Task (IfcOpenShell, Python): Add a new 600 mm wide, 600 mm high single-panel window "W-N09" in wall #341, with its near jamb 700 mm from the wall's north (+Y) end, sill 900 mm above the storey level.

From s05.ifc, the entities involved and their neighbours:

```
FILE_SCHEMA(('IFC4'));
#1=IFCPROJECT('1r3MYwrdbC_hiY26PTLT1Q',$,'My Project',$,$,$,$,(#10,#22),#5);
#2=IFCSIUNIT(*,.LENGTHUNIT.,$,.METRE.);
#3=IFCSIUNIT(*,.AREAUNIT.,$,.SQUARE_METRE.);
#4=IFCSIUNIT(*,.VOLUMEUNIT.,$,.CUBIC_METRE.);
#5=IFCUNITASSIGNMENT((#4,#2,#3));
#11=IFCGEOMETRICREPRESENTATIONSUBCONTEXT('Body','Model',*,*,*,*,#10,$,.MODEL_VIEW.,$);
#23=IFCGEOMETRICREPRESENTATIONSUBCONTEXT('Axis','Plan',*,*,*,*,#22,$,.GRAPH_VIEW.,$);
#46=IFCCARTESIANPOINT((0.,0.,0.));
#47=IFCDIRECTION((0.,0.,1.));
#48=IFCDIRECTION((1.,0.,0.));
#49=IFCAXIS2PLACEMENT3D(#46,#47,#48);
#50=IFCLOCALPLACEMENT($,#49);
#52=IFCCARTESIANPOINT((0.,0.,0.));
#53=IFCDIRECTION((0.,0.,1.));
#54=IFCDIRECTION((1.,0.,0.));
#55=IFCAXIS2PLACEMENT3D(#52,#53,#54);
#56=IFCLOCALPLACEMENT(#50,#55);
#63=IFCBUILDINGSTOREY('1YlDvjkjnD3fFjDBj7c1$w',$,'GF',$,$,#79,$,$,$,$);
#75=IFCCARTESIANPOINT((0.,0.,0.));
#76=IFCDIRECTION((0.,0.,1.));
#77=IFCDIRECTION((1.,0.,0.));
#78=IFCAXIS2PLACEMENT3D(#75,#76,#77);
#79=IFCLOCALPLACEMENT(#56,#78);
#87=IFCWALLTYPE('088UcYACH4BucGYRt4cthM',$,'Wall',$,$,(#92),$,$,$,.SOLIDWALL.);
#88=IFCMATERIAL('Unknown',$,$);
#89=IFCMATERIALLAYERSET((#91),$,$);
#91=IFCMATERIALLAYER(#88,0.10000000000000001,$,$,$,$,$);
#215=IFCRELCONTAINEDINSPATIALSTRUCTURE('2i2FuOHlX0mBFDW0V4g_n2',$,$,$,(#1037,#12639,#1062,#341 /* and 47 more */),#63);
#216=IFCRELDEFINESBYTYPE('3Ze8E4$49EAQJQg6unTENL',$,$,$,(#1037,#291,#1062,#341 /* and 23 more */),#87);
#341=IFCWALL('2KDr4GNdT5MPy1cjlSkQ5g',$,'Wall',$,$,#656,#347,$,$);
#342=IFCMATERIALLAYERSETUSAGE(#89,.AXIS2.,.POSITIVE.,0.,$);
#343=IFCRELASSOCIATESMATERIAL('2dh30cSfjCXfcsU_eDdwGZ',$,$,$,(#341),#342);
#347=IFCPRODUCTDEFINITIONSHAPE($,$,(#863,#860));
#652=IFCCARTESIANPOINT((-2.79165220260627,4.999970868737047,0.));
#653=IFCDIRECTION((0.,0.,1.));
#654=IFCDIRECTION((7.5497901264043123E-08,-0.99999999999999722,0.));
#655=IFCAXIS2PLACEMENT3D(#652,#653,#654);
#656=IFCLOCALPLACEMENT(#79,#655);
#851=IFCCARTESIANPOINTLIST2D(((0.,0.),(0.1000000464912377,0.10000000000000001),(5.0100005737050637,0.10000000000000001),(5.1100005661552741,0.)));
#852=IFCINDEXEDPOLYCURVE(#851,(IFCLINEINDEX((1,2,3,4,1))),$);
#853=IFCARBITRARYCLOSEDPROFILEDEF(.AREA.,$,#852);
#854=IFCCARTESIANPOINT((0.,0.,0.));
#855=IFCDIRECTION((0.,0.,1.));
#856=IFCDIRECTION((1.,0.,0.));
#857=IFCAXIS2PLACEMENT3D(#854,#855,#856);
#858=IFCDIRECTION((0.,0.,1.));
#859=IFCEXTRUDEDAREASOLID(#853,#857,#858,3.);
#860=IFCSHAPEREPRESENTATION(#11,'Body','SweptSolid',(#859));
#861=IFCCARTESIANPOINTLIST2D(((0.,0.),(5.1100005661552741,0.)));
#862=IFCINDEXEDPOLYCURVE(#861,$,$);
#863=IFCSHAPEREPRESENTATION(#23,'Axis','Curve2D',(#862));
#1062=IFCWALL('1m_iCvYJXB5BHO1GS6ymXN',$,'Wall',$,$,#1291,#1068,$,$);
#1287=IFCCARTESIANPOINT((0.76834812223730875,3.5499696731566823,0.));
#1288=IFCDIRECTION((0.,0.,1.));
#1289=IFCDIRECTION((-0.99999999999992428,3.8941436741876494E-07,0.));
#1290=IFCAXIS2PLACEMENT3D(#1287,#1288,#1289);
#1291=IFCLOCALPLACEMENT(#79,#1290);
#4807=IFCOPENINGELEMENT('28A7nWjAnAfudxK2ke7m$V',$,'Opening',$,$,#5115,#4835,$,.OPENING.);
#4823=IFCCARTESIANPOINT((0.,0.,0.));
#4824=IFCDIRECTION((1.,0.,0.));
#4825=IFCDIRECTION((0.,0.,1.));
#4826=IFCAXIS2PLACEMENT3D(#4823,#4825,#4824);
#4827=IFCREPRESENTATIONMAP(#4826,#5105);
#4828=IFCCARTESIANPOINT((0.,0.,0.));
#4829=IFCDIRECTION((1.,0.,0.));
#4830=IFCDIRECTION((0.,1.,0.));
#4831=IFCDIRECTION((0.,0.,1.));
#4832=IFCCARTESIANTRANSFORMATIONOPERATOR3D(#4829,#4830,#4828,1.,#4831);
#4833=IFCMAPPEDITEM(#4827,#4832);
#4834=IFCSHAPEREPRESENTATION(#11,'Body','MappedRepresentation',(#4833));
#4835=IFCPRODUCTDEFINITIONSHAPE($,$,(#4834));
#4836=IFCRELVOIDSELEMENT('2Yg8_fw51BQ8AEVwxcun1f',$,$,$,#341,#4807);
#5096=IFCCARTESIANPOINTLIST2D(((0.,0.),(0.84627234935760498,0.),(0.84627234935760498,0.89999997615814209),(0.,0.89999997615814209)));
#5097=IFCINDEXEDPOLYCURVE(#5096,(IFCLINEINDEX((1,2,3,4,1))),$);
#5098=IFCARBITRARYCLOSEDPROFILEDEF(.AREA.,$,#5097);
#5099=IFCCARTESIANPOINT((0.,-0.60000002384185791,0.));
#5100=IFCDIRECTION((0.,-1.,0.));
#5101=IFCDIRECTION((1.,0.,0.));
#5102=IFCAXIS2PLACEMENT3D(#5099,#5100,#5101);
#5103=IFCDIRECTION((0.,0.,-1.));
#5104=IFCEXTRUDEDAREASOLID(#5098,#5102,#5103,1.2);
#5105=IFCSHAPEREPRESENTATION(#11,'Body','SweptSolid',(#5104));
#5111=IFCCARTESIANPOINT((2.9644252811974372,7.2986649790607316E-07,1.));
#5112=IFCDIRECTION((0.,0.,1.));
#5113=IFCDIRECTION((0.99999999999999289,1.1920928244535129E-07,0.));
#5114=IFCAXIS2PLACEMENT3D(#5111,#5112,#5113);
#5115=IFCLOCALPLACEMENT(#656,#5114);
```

```python
import numpy as np
import ifcopenshell
import ifcopenshell.api.feature
import ifcopenshell.api.geometry
import ifcopenshell.api.root
import ifcopenshell.api.spatial
import ifcopenshell.geom
import ifcopenshell.util.element
import ifcopenshell.util.placement
import ifcopenshell.util.representation
import ifcopenshell.util.shape
import ifcopenshell.util.unit

model = ifcopenshell.open("s05.ifc")
unit_scale = ifcopenshell.util.unit.calculate_unit_scale(model)
settings = ifcopenshell.geom.settings()


def volume(element):
    """Net volume in cubic metres, openings subtracted."""
    shape = ifcopenshell.geom.create_shape(settings, element)
    return ifcopenshell.util.shape.get_volume(shape.geometry)


wall = model.by_guid("2KDr4GNdT5MPy1cjlSkQ5g")
storey = ifcopenshell.util.element.get_container(wall, ifc_class="IfcBuildingStorey")
context = ifcopenshell.util.representation.get_context(model, "Model", "Body", "MODEL_VIEW")
before = volume(wall)

width, height, from_end, sill = 0.6, 0.6, 0.7, 0.9  # metres

# The wall runs along its own X axis, and the end named is its -X end.
wall_shape = ifcopenshell.geom.create_shape(settings, wall)
x, y, z = ifcopenshell.util.shape.get_vertices(wall_shape.geometry).T
start = x.min() + from_end
face, thickness = float(y.min()), float(y.max() - y.min())
wall_matrix = ifcopenshell.util.placement.get_local_placement(wall.ObjectPlacement)
level = ifcopenshell.util.placement.get_local_placement(storey.ObjectPlacement)[2, 3]


def in_wall(x, y):
    """Placement at x, y metres in the wall's axes, at sill height."""
    matrix = wall_matrix.copy()
    matrix[:, 3] = wall_matrix @ np.array([x / unit_scale, y / unit_scale, 0.0, 1.0])
    matrix[2, 3] = level + sill / unit_scale
    return matrix


# Opening: a box that overshoots both wall faces by 50 mm.
opening = ifcopenshell.api.root.create_entity(model, ifc_class="IfcOpeningElement", predefined_type="OPENING")
box = ifcopenshell.api.geometry.add_wall_representation(
    model, context=context, length=width, height=height, thickness=thickness + 0.1
)
ifcopenshell.api.geometry.assign_representation(model, product=opening, representation=box)
ifcopenshell.api.geometry.edit_object_placement(model, product=opening, matrix=in_wall(start, face - 0.05), is_si=False)
ifcopenshell.api.feature.add_feature(model, feature=opening, element=wall)

window = ifcopenshell.api.root.create_entity(model, ifc_class="IfcWindow", name="W-N09", predefined_type="WINDOW")
window.OverallWidth, window.OverallHeight = width / unit_scale, height / unit_scale
window.PartitioningType = "SINGLE_PANEL"
body = ifcopenshell.api.geometry.add_window_representation(
    model,
    context=context,
    overall_width=window.OverallWidth,
    overall_height=window.OverallHeight,
    partition_type="SINGLE_PANEL",
)
ifcopenshell.api.geometry.assign_representation(model, product=window, representation=body)
ifcopenshell.api.spatial.assign_container(model, products=[window], relating_structure=storey)
ifcopenshell.api.feature.add_filling(model, opening=opening, element=window)

# Centre the window in the wall's thickness.
ifcopenshell.api.geometry.edit_object_placement(model, product=window, matrix=in_wall(start, face), is_si=False)
window_shape = ifcopenshell.geom.create_shape(settings, window)
depth = ifcopenshell.util.shape.get_vertices(window_shape.geometry)[:, 1]
offset = face + thickness / 2 - (depth.min() + depth.max()) / 2
ifcopenshell.api.geometry.edit_object_placement(model, product=window, matrix=in_wall(start, offset), is_si=False)

after = volume(wall)

print(f"wall volume {before:.3f} -> {after:.3f} m3")

model.write("s05_updated.ifc")
```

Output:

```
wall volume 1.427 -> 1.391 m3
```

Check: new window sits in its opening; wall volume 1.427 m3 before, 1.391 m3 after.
